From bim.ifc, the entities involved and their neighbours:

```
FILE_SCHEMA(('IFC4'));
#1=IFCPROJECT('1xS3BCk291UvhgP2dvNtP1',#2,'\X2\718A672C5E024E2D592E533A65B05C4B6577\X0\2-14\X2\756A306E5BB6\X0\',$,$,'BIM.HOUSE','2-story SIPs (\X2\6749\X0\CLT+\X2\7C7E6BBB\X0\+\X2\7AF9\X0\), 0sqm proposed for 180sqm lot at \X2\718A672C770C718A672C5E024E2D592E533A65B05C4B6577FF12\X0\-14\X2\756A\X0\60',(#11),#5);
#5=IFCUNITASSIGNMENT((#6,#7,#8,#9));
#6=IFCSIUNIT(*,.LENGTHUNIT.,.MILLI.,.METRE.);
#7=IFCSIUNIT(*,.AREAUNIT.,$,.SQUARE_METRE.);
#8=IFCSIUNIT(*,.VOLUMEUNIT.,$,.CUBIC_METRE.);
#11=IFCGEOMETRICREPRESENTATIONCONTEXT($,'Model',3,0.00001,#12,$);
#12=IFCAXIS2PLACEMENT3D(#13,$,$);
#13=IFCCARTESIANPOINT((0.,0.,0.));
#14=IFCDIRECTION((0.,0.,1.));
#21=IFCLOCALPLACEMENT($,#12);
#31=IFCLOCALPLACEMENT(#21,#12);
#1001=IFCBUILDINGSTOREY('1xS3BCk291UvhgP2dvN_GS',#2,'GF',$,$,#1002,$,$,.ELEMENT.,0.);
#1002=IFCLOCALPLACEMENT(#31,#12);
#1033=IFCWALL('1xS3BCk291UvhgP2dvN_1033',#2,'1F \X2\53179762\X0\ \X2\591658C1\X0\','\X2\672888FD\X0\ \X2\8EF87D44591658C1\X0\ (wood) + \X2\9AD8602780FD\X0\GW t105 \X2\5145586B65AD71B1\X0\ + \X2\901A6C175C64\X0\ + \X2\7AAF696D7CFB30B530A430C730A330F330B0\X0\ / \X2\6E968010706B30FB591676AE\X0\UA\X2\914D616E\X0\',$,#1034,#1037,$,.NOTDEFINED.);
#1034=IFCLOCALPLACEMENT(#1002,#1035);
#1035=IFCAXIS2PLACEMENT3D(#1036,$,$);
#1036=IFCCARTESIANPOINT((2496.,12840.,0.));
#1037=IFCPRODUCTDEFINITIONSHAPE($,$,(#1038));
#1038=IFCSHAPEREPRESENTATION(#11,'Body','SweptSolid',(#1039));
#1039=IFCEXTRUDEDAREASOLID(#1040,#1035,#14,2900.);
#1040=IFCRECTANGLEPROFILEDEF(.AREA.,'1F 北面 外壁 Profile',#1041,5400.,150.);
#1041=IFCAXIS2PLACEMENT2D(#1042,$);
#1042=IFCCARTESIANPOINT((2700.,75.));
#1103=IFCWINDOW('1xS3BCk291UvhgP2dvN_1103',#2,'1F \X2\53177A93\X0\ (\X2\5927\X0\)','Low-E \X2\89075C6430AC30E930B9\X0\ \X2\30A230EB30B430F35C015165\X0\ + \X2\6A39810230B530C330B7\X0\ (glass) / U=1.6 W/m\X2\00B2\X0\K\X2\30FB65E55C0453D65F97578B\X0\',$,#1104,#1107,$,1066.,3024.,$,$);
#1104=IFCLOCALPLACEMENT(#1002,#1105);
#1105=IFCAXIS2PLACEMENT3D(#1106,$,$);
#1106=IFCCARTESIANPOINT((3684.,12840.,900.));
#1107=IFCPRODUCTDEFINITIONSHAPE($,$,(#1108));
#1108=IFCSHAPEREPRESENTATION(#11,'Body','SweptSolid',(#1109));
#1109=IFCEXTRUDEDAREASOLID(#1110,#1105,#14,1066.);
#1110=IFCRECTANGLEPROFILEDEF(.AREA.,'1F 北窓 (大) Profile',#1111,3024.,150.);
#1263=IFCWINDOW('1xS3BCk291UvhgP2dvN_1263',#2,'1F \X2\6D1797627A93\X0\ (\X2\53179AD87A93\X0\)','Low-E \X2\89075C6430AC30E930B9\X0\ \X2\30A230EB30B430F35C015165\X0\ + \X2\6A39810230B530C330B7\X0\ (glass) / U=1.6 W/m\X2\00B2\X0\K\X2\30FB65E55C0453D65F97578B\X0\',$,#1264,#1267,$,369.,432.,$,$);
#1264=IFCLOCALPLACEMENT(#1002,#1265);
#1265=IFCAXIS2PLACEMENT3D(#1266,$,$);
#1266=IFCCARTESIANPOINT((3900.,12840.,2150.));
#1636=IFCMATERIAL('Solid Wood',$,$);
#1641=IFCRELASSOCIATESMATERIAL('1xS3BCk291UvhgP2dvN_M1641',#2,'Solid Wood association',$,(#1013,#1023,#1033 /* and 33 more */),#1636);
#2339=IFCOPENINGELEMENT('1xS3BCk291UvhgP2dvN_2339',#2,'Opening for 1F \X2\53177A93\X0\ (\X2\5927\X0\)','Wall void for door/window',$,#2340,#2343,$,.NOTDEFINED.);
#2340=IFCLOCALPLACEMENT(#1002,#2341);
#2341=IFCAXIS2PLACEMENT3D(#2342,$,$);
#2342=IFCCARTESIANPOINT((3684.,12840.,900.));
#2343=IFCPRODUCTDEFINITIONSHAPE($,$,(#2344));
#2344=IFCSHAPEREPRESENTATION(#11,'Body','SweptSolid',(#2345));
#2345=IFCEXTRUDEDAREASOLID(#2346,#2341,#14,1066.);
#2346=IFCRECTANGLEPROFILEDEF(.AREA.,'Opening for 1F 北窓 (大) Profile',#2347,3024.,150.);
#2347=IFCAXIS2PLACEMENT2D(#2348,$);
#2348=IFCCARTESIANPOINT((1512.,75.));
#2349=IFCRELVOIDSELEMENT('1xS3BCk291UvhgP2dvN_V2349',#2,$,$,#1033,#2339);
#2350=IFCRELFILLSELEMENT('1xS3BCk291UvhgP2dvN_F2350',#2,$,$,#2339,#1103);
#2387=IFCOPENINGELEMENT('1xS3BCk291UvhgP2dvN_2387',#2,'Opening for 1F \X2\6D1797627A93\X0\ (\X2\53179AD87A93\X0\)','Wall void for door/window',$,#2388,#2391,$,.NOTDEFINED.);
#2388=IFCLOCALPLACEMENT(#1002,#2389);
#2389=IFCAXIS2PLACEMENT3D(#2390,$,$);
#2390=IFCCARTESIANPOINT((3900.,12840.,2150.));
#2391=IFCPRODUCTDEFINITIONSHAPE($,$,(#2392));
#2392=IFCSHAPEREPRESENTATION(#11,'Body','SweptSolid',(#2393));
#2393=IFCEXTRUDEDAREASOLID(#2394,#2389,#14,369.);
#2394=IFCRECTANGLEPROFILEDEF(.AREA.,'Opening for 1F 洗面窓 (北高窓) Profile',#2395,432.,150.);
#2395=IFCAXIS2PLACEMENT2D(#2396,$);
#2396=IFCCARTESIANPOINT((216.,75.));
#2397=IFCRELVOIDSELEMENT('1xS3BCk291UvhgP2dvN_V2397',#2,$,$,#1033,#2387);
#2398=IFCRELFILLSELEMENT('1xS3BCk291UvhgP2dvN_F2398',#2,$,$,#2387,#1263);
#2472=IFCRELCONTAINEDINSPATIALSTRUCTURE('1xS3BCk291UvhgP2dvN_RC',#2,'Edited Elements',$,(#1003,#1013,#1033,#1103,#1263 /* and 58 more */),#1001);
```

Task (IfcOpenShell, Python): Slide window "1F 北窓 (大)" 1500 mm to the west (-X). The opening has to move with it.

```python
import ifcopenshell
import ifcopenshell.api.geometry
import ifcopenshell.util.placement
import ifcopenshell.util.unit

model = ifcopenshell.open("bim.ifc")
unit_scale = ifcopenshell.util.unit.calculate_unit_scale(model)

window = model.by_guid("1xS3BCk291UvhgP2dvN_1103")
opening = window.FillsVoids[0].RelatingOpeningElement
wall = opening.VoidsElements[0].RelatingBuildingElement

wall_matrix = ifcopenshell.util.placement.get_local_placement(wall.ObjectPlacement)
shift = wall_matrix[:3, 0] * -1.5 / unit_scale
before = ifcopenshell.util.placement.get_local_placement(window.ObjectPlacement)[:3, 3].copy()

# The window is not placed relative to its opening, so move both.
for product in (opening, window):
    matrix = ifcopenshell.util.placement.get_local_placement(product.ObjectPlacement)
    matrix[:3, 3] += shift
    ifcopenshell.api.geometry.edit_object_placement(model, product=product, matrix=matrix, is_si=False)

after = ifcopenshell.util.placement.get_local_placement(window.ObjectPlacement)[:3, 3]
print("window moved by", (after - before).round(3) + 0.0)

model.write("bim_updated.ifc")
```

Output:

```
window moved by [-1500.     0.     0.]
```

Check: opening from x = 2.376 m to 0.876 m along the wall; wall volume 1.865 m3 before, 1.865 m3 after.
